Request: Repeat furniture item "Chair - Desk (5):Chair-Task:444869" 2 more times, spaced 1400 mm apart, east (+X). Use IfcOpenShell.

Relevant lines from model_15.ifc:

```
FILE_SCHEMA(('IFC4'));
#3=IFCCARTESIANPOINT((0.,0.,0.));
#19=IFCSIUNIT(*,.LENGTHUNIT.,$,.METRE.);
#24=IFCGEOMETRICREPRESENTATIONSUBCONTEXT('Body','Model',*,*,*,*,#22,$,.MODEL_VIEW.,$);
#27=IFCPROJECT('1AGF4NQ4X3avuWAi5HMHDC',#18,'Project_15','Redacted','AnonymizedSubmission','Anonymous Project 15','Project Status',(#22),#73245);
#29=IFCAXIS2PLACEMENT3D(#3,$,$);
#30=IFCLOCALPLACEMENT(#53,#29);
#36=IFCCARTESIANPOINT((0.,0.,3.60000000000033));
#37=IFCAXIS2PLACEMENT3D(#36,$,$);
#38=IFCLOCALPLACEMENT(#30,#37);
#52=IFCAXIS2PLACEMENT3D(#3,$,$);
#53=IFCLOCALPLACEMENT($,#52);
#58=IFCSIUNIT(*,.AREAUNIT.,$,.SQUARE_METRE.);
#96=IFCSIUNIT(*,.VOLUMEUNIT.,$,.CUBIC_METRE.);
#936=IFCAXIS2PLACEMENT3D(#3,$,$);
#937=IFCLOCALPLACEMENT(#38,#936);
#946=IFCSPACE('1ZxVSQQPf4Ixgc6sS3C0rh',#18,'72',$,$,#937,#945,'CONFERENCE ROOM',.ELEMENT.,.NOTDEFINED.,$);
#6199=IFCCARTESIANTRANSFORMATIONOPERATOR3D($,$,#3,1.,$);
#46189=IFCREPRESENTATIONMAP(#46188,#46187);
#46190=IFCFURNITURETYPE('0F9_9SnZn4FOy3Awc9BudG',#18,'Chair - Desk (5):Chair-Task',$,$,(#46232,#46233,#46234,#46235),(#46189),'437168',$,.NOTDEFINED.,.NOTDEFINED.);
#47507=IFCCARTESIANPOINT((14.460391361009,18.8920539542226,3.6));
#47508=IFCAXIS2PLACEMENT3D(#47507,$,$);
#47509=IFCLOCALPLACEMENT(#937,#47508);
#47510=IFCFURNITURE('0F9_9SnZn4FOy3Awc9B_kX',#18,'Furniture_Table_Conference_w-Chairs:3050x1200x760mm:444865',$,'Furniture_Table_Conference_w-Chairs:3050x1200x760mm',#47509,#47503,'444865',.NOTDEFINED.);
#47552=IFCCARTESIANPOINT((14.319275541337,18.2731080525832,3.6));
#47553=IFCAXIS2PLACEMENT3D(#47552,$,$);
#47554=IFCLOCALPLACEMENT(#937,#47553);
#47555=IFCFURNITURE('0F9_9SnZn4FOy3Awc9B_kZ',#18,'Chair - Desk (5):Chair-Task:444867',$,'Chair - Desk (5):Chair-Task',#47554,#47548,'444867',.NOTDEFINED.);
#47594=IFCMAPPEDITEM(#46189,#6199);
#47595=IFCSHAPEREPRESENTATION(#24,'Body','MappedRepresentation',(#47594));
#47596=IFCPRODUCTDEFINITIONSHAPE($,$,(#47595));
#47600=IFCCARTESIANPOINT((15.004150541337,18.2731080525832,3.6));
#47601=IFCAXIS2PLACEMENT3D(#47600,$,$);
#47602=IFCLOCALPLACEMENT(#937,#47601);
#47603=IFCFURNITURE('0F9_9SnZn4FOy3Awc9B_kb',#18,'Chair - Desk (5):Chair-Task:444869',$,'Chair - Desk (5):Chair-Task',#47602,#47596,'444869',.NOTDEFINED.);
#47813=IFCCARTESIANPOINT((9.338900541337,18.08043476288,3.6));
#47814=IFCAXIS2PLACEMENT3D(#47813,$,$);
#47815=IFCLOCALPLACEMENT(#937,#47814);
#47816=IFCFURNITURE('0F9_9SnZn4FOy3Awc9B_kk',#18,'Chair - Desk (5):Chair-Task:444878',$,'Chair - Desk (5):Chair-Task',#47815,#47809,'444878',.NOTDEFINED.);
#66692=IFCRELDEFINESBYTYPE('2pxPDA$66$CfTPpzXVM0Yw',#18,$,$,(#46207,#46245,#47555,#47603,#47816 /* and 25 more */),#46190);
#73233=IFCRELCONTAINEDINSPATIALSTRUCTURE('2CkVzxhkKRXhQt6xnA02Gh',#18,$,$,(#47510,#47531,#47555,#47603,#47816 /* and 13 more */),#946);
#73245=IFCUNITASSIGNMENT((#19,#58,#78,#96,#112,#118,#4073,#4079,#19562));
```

```python
import numpy as np
import ifcopenshell
import ifcopenshell.api.geometry
import ifcopenshell.api.root
import ifcopenshell.util.element
import ifcopenshell.util.placement
import ifcopenshell.util.unit

model = ifcopenshell.open("model_15.ifc")
unit_scale = ifcopenshell.util.unit.calculate_unit_scale(model)


def reuse_history(source, copy):
    """copy_class also copies each property set's owner history, people and application; keep the originals."""
    for rel in copy.IsDefinedBy:
        if rel.is_a("IfcRelDefinesByProperties") and (history := rel.RelatingPropertyDefinition.OwnerHistory):
            rel.RelatingPropertyDefinition.OwnerHistory = source.OwnerHistory
            ifcopenshell.util.element.remove_deep2(model, history)


source = model.by_id(47603)
base = ifcopenshell.util.placement.get_local_placement(source.ObjectPlacement)
step = np.array([1.0, 0.0, 0.0]) * 1.4 / unit_scale

for i in range(1, 3):
    copy = ifcopenshell.api.root.copy_class(model, product=source)
    copy.Representation = ifcopenshell.util.element.copy_deep(
        model, source.Representation, exclude=["IfcGeometricRepresentationContext", "IfcRepresentationMap"]
    )
    copy.Name = "Chair - Desk (5):Chair-Task"
    copy.Tag = None
    reuse_history(source, copy)
    matrix = base.copy()
    matrix[:3, 3] += i * step
    print("added at", matrix[:3, 3].round(3) + 0.0)
    ifcopenshell.api.geometry.edit_object_placement(model, product=copy, matrix=matrix, is_si=False)

model.write("model_15_edited.ifc")
```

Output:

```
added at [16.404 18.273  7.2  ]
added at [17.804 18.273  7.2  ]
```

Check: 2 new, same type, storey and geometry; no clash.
